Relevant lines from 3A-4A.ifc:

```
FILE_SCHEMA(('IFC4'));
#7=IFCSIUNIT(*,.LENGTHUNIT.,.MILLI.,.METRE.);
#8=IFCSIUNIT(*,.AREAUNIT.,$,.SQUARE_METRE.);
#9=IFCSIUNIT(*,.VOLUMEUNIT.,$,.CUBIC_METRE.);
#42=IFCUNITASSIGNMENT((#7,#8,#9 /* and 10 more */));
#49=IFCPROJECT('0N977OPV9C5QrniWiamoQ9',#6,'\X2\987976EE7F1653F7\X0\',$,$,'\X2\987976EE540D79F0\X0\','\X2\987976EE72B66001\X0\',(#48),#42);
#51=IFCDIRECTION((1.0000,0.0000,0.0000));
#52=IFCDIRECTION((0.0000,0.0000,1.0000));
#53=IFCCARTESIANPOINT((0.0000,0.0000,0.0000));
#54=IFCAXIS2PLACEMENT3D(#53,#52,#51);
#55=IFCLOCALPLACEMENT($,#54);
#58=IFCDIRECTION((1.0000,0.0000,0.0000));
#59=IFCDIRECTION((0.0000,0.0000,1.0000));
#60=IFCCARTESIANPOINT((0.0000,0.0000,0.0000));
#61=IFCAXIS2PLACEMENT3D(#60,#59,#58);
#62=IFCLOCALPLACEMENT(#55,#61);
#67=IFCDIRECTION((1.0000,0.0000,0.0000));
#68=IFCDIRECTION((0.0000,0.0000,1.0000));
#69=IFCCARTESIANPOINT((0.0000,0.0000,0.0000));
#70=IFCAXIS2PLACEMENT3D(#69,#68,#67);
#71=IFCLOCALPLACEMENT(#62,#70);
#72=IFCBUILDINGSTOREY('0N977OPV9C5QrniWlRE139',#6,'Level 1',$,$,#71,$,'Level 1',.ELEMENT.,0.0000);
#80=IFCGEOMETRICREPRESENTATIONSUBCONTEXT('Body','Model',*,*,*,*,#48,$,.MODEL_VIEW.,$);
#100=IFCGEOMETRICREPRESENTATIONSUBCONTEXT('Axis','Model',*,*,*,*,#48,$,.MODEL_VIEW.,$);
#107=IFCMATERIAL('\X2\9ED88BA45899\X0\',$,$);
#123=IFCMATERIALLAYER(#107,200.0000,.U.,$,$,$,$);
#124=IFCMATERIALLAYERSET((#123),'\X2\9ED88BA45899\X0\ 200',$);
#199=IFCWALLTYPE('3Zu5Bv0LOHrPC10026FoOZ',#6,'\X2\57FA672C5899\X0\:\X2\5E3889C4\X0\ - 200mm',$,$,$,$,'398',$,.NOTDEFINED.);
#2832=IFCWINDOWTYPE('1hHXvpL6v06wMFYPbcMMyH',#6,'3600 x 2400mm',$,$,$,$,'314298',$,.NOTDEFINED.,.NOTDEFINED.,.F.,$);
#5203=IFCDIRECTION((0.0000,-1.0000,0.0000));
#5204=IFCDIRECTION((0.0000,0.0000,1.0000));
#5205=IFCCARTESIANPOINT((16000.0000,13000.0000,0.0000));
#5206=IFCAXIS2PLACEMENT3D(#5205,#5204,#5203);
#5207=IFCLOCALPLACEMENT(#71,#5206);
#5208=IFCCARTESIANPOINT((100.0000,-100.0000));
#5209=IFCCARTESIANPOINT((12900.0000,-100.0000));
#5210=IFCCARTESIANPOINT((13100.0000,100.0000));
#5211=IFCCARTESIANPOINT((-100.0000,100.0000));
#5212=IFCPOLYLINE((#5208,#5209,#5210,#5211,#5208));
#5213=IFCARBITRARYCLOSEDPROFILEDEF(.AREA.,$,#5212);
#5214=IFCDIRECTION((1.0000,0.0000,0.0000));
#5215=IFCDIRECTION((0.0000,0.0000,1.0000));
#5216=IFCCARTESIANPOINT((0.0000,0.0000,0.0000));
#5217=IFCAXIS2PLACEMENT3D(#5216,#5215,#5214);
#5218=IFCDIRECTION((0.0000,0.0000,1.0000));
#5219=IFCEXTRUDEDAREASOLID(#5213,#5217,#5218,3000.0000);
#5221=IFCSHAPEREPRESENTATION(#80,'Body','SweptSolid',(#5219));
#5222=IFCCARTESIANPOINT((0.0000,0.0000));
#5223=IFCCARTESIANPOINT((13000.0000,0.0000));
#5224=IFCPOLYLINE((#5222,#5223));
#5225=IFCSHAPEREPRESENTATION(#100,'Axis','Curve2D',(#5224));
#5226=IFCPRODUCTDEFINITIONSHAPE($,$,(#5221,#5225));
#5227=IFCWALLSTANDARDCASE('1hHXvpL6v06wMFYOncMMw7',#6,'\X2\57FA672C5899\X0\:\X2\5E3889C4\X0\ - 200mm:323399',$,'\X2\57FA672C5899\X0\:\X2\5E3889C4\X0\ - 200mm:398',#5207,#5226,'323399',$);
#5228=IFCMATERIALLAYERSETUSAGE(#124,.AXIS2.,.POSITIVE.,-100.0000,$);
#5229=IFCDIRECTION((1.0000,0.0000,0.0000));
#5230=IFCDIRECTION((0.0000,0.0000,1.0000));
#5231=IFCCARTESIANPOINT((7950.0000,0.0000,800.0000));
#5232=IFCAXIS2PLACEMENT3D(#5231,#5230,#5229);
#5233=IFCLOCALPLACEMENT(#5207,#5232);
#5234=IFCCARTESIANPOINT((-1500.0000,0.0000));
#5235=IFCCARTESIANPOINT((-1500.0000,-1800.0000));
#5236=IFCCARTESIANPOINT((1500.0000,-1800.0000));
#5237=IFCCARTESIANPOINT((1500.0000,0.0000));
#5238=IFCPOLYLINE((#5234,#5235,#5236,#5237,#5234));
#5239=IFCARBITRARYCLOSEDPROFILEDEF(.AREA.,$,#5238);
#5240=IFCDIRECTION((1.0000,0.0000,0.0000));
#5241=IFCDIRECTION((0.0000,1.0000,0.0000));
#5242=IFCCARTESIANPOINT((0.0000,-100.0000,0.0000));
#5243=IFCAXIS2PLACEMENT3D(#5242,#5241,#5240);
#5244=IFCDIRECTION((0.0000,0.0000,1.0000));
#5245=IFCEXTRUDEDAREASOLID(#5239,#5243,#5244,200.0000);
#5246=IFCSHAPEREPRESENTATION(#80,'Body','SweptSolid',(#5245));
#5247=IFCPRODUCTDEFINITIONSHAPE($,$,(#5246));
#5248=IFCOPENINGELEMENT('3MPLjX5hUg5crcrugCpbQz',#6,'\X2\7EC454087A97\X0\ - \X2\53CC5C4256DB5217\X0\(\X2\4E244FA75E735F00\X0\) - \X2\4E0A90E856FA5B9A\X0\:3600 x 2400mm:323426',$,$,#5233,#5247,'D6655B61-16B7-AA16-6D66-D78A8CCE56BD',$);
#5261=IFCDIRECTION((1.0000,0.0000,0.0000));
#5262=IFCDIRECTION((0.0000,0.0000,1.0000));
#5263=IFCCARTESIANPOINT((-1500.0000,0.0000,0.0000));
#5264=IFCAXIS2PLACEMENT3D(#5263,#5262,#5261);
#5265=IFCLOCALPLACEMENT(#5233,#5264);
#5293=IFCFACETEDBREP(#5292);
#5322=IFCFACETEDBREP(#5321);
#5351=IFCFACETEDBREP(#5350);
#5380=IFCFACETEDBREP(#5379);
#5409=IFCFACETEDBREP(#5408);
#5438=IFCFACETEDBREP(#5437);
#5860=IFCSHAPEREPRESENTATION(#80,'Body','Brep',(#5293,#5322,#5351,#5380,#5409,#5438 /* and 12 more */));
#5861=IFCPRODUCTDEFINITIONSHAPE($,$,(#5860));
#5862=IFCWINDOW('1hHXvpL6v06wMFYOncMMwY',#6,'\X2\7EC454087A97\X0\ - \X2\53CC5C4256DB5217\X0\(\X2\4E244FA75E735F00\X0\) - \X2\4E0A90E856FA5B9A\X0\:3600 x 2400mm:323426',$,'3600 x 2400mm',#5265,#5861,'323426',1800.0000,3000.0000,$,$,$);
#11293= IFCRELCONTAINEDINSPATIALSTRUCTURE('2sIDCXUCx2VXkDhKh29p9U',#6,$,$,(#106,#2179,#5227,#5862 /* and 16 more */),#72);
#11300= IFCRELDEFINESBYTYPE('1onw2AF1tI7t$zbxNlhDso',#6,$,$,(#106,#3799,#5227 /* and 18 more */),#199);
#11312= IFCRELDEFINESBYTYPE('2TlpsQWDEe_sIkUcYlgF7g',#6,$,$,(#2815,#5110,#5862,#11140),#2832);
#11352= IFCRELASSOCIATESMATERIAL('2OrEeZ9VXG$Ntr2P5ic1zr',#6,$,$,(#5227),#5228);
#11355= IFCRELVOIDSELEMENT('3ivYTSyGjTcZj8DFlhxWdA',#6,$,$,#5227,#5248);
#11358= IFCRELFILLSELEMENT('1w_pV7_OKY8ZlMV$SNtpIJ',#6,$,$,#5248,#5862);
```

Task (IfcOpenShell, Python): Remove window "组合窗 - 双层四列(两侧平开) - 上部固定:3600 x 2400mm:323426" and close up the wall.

```python
import ifcopenshell
import ifcopenshell.api.feature
import ifcopenshell.api.root
import ifcopenshell.geom
import ifcopenshell.util.shape

model = ifcopenshell.open("3A-4A.ifc")
settings = ifcopenshell.geom.settings()


def volume(element):
    """Net volume in cubic metres, openings subtracted."""
    shape = ifcopenshell.geom.create_shape(settings, element)
    return ifcopenshell.util.shape.get_volume(shape.geometry)


window = model.by_id(5862)
opening = window.FillsVoids[0].RelatingOpeningElement
wall = opening.VoidsElements[0].RelatingBuildingElement
before = volume(wall)

ifcopenshell.api.root.remove_product(model, product=window)
ifcopenshell.api.feature.remove_feature(model, feature=opening)

after = volume(wall)

print(f"wall volume {before:.3f} -> {after:.3f} m3")

model.write("3A-4A_edited.ifc")
```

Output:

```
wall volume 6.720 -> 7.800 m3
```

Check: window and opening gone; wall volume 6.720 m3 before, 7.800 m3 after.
